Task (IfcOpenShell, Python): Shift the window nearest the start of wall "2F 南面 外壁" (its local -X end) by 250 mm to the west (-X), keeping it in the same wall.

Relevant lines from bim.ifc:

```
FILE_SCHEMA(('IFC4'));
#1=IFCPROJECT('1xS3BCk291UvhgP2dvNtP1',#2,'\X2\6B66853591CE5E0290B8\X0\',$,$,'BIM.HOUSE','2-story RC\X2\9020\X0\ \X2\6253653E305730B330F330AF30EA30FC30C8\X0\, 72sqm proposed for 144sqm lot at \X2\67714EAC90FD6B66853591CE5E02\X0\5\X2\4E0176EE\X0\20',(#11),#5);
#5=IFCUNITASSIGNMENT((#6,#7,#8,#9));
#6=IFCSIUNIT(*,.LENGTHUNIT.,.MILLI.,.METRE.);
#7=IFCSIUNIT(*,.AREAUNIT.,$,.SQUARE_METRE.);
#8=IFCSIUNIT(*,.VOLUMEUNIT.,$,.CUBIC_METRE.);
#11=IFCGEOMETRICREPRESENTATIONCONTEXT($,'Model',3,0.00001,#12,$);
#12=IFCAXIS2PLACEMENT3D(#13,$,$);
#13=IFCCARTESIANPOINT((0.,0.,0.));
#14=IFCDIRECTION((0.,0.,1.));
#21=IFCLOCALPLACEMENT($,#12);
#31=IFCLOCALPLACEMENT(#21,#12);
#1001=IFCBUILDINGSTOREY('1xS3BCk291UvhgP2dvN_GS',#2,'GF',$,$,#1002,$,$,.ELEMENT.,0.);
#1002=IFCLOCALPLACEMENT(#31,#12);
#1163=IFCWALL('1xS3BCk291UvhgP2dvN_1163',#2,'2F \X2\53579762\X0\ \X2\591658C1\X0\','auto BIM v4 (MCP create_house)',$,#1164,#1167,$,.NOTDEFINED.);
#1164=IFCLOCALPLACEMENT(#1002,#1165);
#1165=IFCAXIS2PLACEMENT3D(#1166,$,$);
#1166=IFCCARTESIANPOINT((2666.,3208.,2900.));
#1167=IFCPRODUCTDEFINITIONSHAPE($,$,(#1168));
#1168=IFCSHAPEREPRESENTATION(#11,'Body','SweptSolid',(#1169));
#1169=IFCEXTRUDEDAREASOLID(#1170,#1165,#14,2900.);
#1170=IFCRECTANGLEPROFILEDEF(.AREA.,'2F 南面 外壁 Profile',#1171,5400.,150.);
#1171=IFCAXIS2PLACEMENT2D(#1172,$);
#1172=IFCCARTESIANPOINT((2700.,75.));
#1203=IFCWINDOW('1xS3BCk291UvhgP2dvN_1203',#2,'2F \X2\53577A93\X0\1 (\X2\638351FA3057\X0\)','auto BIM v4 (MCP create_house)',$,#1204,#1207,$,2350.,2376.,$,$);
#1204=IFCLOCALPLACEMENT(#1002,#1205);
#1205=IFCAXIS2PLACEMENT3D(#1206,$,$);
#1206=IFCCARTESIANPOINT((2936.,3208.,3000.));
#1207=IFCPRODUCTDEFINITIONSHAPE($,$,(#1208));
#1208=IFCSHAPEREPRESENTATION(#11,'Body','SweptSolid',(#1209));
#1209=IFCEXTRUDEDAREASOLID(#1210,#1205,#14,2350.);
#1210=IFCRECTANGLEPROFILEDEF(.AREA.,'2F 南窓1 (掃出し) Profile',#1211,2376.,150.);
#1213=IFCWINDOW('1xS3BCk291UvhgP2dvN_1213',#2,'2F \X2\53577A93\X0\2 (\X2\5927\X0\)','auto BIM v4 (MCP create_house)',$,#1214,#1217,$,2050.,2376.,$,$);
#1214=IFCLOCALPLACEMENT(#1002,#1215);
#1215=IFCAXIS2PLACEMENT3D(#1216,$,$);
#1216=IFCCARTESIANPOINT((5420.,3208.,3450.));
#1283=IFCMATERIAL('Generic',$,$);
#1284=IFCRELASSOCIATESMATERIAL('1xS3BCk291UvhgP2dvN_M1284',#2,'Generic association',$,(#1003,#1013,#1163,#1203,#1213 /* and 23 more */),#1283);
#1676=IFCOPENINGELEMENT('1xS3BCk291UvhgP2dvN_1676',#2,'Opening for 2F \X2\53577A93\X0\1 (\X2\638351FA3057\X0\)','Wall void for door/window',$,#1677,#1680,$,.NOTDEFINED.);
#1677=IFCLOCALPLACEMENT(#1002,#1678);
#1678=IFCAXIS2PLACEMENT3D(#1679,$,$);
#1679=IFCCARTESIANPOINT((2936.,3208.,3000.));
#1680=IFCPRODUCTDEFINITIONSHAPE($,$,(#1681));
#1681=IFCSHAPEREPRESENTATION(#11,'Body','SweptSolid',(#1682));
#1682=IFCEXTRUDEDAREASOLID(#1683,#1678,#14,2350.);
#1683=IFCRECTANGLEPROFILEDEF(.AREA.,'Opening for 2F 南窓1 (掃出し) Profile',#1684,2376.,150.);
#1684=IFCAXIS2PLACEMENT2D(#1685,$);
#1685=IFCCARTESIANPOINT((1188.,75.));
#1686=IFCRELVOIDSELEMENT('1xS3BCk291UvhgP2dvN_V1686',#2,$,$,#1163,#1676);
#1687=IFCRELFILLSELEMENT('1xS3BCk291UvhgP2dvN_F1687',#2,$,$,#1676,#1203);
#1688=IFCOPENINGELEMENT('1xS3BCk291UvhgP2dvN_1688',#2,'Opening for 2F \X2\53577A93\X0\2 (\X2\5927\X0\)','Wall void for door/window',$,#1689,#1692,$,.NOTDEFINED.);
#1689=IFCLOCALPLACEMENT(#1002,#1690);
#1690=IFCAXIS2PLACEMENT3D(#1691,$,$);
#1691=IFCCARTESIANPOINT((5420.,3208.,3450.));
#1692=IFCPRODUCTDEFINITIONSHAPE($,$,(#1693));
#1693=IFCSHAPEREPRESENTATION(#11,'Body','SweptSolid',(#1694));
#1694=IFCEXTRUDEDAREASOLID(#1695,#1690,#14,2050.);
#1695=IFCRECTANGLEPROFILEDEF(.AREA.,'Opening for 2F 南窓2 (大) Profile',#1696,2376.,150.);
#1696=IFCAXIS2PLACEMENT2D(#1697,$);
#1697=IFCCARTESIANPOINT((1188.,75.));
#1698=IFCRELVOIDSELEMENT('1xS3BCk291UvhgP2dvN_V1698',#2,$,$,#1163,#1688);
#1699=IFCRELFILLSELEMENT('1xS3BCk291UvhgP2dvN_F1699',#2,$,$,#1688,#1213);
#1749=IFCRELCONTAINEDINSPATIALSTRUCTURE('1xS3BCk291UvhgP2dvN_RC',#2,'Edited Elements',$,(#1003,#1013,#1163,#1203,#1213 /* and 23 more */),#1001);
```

```python
import ifcopenshell
import ifcopenshell.api.geometry
import ifcopenshell.util.placement
import ifcopenshell.util.unit

model = ifcopenshell.open("bim.ifc")
unit_scale = ifcopenshell.util.unit.calculate_unit_scale(model)

window = model.by_id(1203)
opening = window.FillsVoids[0].RelatingOpeningElement
wall = opening.VoidsElements[0].RelatingBuildingElement

wall_matrix = ifcopenshell.util.placement.get_local_placement(wall.ObjectPlacement)
shift = wall_matrix[:3, 0] * -0.25 / unit_scale
before = ifcopenshell.util.placement.get_local_placement(window.ObjectPlacement)[:3, 3].copy()

# The window is not placed relative to its opening, so move both.
for product in (opening, window):
    matrix = ifcopenshell.util.placement.get_local_placement(product.ObjectPlacement)
    matrix[:3, 3] += shift
    ifcopenshell.api.geometry.edit_object_placement(model, product=product, matrix=matrix, is_si=False)

after = ifcopenshell.util.placement.get_local_placement(window.ObjectPlacement)[:3, 3]
print("window moved by", (after - before).round(3) + 0.0)

model.write("bim_edited.ifc")
```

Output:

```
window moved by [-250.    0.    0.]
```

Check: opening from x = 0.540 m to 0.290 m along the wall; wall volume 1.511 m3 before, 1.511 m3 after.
